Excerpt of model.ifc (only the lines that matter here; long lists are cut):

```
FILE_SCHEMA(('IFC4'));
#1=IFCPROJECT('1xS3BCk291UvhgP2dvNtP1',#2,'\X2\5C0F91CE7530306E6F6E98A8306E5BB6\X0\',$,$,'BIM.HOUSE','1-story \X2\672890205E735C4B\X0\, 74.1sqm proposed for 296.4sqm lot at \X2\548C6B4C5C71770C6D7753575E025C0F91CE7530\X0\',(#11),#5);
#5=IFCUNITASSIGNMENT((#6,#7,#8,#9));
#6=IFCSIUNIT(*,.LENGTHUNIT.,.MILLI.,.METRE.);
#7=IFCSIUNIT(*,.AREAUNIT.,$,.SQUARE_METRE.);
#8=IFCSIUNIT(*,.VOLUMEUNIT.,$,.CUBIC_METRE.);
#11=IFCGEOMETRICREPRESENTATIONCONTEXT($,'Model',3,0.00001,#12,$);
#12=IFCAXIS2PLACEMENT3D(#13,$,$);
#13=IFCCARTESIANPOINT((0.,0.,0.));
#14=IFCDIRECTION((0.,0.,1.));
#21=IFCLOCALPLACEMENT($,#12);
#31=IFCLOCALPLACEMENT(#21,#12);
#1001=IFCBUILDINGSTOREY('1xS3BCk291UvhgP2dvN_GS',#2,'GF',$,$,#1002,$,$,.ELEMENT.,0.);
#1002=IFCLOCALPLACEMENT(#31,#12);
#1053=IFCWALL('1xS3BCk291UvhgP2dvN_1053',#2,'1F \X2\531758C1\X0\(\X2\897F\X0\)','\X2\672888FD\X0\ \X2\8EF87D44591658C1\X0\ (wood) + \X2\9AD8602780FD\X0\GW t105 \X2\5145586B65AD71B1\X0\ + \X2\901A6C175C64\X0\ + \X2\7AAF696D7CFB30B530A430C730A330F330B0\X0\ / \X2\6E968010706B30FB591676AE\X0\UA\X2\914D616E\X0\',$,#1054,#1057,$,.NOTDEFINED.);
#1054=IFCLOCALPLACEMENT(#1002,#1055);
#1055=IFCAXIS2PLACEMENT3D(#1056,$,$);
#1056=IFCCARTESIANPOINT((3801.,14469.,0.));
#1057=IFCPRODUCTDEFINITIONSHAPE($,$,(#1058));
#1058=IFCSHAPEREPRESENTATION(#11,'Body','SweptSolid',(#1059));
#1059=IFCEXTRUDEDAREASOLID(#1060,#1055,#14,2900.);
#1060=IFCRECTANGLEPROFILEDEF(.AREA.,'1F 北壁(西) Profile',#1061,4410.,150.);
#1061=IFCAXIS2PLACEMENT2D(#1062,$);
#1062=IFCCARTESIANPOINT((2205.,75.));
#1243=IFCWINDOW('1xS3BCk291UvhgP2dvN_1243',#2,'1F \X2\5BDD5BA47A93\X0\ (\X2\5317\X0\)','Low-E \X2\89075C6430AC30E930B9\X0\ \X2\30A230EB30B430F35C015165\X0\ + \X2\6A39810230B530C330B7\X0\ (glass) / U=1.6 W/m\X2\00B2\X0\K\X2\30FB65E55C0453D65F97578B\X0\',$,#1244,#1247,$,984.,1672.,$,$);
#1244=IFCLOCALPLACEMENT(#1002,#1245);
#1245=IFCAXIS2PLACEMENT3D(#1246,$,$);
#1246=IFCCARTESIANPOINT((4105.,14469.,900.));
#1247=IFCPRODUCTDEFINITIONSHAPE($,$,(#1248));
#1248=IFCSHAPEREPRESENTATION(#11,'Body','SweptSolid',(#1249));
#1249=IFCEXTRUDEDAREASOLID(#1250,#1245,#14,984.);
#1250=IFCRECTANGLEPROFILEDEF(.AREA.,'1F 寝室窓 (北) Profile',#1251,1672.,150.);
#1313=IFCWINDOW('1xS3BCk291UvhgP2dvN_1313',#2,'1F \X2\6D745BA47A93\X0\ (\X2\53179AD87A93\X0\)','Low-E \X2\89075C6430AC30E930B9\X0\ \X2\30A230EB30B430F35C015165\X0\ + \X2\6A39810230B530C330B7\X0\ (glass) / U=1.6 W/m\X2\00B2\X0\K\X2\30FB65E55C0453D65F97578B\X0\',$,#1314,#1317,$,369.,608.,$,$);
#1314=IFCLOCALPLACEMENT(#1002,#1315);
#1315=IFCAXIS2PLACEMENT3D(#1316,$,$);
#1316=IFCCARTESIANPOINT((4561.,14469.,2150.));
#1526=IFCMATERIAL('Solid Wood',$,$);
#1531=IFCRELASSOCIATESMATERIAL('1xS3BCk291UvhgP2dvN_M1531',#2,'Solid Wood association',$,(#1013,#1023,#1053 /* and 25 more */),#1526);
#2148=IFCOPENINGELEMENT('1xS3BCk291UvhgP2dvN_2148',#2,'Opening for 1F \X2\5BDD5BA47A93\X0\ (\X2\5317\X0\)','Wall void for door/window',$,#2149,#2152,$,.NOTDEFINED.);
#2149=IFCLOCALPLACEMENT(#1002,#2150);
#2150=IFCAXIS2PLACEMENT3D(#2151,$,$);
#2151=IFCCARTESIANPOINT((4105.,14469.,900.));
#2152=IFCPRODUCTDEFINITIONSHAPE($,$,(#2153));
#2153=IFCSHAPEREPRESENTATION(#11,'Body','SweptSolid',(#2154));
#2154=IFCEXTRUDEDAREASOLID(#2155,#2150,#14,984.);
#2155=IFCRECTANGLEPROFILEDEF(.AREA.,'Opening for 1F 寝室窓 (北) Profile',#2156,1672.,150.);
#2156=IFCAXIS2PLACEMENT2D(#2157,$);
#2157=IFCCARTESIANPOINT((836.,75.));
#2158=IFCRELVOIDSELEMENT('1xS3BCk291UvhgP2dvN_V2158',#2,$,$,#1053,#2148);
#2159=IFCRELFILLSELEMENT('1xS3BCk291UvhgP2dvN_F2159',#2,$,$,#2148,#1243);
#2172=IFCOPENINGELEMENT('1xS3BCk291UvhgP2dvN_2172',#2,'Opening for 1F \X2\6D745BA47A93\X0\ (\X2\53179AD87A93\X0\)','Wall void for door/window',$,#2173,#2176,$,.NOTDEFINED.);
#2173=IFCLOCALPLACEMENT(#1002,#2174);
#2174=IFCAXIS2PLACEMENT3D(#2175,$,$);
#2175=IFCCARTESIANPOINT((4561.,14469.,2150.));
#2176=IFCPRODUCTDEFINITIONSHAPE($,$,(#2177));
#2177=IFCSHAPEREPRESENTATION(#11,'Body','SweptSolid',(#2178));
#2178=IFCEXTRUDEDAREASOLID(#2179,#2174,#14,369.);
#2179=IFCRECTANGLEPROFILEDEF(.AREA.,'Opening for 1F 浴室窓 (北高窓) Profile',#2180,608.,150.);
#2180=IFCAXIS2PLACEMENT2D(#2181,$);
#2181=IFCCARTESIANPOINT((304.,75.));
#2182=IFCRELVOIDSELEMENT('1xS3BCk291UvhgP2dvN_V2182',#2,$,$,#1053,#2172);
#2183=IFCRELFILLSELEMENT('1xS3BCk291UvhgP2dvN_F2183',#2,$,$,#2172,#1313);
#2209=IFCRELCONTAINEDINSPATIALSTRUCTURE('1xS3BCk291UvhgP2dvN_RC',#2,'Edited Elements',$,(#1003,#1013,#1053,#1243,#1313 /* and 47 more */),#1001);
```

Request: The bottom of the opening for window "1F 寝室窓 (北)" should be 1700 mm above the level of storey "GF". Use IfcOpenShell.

```python
import numpy as np
import ifcopenshell
import ifcopenshell.api.geometry
import ifcopenshell.geom
import ifcopenshell.util.element
import ifcopenshell.util.placement
import ifcopenshell.util.shape
import ifcopenshell.util.unit

model = ifcopenshell.open("model.ifc")
unit_scale = ifcopenshell.util.unit.calculate_unit_scale(model)

window = model.by_guid("1xS3BCk291UvhgP2dvN_1243")
opening = window.FillsVoids[0].RelatingOpeningElement
storey = ifcopenshell.util.element.get_container(window, ifc_class="IfcBuildingStorey")
level = ifcopenshell.util.placement.get_local_placement(storey.ObjectPlacement)[2, 3]

# The opening's origin need not be at the sill, so measure its lowest point.
shape = ifcopenshell.geom.create_shape(ifcopenshell.geom.settings(), opening)
bottom = ifcopenshell.util.shape.get_shape_bottom_elevation(shape, shape.geometry) / unit_scale
dz = level + 1.7 / unit_scale - bottom

shift = np.array([0.0, 0.0, dz])
# The window is not placed relative to its opening, so move both.
for product in (opening, window):
    matrix = ifcopenshell.util.placement.get_local_placement(product.ObjectPlacement)
    matrix[:3, 3] += shift
    ifcopenshell.api.geometry.edit_object_placement(model, product=product, matrix=matrix, is_si=False)

print(f"moved by {dz * unit_scale:+.3f} m")

model.write("model_edited.ifc")
```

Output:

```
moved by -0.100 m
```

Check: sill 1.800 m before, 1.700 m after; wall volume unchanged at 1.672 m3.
